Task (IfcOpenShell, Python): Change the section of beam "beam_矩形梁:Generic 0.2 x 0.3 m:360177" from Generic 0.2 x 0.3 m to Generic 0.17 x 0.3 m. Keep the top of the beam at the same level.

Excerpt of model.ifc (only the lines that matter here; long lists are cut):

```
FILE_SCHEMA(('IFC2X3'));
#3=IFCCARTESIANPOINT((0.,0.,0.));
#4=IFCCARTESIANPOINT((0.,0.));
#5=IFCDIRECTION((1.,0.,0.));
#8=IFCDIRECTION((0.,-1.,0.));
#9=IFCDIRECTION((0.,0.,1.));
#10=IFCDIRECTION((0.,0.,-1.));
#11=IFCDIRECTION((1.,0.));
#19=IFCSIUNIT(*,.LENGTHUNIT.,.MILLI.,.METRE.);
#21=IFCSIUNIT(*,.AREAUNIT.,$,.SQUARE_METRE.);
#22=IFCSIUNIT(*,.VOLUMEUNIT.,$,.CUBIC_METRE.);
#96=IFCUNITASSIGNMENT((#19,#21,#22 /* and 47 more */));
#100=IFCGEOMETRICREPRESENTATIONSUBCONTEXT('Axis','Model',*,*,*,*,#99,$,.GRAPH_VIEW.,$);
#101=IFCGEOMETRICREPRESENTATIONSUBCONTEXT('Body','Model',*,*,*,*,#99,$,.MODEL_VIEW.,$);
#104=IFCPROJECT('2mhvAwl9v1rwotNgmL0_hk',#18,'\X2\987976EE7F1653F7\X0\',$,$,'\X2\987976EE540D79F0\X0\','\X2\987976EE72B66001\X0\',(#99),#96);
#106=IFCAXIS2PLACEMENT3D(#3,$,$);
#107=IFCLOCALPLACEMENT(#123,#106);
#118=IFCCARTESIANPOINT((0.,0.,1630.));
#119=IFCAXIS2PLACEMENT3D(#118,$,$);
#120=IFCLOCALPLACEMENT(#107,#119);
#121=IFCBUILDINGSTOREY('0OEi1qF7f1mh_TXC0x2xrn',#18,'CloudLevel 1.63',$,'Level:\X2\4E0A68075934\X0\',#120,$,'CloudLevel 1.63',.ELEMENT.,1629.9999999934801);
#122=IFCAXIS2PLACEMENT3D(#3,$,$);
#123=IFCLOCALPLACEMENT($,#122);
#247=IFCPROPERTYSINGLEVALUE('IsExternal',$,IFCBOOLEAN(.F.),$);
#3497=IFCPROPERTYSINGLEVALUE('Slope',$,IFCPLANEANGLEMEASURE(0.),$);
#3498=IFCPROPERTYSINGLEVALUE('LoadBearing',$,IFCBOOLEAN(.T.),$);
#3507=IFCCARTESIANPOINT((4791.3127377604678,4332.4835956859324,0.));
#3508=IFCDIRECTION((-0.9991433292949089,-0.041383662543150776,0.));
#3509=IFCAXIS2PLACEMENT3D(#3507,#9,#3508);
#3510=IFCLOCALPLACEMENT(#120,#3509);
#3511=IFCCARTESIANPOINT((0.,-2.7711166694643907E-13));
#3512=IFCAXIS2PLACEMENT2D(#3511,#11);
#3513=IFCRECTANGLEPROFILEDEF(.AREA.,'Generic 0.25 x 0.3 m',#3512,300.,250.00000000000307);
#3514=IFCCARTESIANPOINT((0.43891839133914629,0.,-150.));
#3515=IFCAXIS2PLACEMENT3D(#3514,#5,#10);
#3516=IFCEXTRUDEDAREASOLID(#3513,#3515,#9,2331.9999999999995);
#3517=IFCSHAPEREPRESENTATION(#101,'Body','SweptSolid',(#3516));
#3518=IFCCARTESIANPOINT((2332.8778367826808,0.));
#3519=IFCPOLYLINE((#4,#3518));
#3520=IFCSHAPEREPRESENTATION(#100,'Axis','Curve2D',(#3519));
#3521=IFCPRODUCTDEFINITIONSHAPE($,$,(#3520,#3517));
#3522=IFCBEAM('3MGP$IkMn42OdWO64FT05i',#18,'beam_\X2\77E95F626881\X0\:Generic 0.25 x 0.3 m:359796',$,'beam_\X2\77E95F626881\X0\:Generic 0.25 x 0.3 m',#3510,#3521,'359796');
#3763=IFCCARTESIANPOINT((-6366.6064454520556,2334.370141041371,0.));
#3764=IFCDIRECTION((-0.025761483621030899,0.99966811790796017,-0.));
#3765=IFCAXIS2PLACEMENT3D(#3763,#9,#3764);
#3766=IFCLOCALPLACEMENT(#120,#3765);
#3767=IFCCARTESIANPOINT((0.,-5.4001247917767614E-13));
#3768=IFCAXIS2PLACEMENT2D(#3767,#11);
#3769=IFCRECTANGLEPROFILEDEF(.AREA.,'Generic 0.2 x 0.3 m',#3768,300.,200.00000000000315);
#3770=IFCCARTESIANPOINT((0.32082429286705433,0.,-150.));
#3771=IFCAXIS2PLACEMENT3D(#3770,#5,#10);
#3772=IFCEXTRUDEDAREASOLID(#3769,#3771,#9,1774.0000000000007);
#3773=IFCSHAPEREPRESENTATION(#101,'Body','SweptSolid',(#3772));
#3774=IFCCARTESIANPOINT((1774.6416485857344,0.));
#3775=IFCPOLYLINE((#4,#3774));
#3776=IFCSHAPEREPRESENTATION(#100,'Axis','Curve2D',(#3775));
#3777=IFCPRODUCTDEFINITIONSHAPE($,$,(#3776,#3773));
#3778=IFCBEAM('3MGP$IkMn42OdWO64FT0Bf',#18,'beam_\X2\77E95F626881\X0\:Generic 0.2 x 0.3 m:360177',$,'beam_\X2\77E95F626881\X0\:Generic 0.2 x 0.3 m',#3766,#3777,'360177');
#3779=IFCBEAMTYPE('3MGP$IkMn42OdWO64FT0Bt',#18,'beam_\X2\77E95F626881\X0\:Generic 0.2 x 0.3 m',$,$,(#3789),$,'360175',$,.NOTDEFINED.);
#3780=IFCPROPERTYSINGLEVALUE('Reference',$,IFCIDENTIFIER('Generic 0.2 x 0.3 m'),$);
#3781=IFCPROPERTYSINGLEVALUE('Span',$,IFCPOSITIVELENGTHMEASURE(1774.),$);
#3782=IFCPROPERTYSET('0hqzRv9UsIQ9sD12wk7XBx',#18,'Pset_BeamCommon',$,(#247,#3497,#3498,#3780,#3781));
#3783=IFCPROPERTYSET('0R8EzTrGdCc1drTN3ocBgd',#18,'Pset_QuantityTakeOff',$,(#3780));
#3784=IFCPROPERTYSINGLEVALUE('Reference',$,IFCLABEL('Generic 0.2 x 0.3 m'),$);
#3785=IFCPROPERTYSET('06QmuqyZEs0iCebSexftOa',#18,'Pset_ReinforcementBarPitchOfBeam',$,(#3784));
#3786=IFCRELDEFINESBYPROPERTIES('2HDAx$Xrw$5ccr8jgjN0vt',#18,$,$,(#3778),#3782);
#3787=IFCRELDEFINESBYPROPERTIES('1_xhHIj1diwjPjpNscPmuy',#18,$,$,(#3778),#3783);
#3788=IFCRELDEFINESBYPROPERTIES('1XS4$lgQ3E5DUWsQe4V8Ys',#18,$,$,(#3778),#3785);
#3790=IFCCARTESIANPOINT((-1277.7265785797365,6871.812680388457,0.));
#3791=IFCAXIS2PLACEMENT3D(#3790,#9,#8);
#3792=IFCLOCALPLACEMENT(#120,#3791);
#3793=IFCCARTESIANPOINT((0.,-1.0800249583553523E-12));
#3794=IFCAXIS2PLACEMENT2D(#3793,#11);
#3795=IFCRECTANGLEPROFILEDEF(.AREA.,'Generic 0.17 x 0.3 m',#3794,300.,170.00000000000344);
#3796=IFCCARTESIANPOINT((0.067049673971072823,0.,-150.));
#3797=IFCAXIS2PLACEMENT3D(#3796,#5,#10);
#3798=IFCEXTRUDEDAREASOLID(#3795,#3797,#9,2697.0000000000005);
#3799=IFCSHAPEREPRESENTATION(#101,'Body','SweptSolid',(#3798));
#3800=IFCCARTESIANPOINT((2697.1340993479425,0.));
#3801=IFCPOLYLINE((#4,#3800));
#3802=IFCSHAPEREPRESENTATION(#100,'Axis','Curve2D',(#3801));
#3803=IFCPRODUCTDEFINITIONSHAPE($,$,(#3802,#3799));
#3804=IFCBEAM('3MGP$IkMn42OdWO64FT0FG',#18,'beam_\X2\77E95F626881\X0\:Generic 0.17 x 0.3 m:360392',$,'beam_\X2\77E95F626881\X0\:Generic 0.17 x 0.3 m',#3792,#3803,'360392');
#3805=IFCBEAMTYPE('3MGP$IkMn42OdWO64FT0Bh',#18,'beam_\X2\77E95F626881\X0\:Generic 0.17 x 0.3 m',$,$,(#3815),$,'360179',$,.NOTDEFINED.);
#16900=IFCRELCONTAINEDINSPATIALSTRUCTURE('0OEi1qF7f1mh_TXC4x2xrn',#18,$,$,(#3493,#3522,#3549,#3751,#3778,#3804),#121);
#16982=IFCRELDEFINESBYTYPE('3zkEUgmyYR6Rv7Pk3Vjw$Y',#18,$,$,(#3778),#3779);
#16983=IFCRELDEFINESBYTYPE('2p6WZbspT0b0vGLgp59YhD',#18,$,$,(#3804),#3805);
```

```python
import ifcopenshell
import ifcopenshell.api.pset
import ifcopenshell.api.type
import ifcopenshell.util.element
import ifcopenshell.util.representation

model = ifcopenshell.open("model.ifc")

member = model.by_guid("3MGP$IkMn42OdWO64FT0Bf")
source = next(p for p in model.by_type("IfcRectangleProfileDef") if p.ProfileName == "Generic 0.17 x 0.3 m")

body = ifcopenshell.util.representation.get_representation(member, "Model", "Body")
solid = body.Items[0]
old_profile = solid.SweptArea

# Copy the section's sizes but keep this member's own profile position.
profile = ifcopenshell.util.element.copy(model, source)
# Profiles are centred, so shift by half the change in depth to hold the top.
shift = (old_profile.XDim - profile.XDim) / 2
x, y = old_profile.Position.Location.Coordinates
up = (-1.0, 0.0)  # upwards, in the solid's own plane
location = model.createIfcCartesianPoint((x + up[0] * shift, y + up[1] * shift))
profile.Position = model.createIfcAxis2Placement2D(location, old_profile.Position.RefDirection)
solid.SweptArea = profile
if not model.get_total_inverses(old_profile):
    ifcopenshell.util.element.remove_deep2(model, old_profile)

new_type = model.by_guid("3MGP$IkMn42OdWO64FT0Bh")
ifcopenshell.api.type.assign_type(
    model, related_objects=[member], relating_type=new_type, should_map_representations=False
)
member.Name = member.Name.replace("Generic 0.2 x 0.3 m", "Generic 0.17 x 0.3 m")
member.ObjectType = "beam_矩形梁:Generic 0.17 x 0.3 m"
pset = model.by_id(ifcopenshell.util.element.get_pset(member, "Pset_BeamCommon", should_inherit=False)["id"])
ifcopenshell.api.pset.edit_pset(model, pset=pset, properties={"Reference": "Generic 0.17 x 0.3 m"})
pset = model.by_id(ifcopenshell.util.element.get_pset(member, "Pset_QuantityTakeOff", should_inherit=False)["id"])
ifcopenshell.api.pset.edit_pset(model, pset=pset, properties={"Reference": "Generic 0.17 x 0.3 m"})
pset = model.by_id(ifcopenshell.util.element.get_pset(member, "Pset_ReinforcementBarPitchOfBeam", should_inherit=False)["id"])
ifcopenshell.api.pset.edit_pset(model, pset=pset, properties={"Reference": "Generic 0.17 x 0.3 m"})

print(solid.SweptArea)

model.write("model_updated.ifc")
```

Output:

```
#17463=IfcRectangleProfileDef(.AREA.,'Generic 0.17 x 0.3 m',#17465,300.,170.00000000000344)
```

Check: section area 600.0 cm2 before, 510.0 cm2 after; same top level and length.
